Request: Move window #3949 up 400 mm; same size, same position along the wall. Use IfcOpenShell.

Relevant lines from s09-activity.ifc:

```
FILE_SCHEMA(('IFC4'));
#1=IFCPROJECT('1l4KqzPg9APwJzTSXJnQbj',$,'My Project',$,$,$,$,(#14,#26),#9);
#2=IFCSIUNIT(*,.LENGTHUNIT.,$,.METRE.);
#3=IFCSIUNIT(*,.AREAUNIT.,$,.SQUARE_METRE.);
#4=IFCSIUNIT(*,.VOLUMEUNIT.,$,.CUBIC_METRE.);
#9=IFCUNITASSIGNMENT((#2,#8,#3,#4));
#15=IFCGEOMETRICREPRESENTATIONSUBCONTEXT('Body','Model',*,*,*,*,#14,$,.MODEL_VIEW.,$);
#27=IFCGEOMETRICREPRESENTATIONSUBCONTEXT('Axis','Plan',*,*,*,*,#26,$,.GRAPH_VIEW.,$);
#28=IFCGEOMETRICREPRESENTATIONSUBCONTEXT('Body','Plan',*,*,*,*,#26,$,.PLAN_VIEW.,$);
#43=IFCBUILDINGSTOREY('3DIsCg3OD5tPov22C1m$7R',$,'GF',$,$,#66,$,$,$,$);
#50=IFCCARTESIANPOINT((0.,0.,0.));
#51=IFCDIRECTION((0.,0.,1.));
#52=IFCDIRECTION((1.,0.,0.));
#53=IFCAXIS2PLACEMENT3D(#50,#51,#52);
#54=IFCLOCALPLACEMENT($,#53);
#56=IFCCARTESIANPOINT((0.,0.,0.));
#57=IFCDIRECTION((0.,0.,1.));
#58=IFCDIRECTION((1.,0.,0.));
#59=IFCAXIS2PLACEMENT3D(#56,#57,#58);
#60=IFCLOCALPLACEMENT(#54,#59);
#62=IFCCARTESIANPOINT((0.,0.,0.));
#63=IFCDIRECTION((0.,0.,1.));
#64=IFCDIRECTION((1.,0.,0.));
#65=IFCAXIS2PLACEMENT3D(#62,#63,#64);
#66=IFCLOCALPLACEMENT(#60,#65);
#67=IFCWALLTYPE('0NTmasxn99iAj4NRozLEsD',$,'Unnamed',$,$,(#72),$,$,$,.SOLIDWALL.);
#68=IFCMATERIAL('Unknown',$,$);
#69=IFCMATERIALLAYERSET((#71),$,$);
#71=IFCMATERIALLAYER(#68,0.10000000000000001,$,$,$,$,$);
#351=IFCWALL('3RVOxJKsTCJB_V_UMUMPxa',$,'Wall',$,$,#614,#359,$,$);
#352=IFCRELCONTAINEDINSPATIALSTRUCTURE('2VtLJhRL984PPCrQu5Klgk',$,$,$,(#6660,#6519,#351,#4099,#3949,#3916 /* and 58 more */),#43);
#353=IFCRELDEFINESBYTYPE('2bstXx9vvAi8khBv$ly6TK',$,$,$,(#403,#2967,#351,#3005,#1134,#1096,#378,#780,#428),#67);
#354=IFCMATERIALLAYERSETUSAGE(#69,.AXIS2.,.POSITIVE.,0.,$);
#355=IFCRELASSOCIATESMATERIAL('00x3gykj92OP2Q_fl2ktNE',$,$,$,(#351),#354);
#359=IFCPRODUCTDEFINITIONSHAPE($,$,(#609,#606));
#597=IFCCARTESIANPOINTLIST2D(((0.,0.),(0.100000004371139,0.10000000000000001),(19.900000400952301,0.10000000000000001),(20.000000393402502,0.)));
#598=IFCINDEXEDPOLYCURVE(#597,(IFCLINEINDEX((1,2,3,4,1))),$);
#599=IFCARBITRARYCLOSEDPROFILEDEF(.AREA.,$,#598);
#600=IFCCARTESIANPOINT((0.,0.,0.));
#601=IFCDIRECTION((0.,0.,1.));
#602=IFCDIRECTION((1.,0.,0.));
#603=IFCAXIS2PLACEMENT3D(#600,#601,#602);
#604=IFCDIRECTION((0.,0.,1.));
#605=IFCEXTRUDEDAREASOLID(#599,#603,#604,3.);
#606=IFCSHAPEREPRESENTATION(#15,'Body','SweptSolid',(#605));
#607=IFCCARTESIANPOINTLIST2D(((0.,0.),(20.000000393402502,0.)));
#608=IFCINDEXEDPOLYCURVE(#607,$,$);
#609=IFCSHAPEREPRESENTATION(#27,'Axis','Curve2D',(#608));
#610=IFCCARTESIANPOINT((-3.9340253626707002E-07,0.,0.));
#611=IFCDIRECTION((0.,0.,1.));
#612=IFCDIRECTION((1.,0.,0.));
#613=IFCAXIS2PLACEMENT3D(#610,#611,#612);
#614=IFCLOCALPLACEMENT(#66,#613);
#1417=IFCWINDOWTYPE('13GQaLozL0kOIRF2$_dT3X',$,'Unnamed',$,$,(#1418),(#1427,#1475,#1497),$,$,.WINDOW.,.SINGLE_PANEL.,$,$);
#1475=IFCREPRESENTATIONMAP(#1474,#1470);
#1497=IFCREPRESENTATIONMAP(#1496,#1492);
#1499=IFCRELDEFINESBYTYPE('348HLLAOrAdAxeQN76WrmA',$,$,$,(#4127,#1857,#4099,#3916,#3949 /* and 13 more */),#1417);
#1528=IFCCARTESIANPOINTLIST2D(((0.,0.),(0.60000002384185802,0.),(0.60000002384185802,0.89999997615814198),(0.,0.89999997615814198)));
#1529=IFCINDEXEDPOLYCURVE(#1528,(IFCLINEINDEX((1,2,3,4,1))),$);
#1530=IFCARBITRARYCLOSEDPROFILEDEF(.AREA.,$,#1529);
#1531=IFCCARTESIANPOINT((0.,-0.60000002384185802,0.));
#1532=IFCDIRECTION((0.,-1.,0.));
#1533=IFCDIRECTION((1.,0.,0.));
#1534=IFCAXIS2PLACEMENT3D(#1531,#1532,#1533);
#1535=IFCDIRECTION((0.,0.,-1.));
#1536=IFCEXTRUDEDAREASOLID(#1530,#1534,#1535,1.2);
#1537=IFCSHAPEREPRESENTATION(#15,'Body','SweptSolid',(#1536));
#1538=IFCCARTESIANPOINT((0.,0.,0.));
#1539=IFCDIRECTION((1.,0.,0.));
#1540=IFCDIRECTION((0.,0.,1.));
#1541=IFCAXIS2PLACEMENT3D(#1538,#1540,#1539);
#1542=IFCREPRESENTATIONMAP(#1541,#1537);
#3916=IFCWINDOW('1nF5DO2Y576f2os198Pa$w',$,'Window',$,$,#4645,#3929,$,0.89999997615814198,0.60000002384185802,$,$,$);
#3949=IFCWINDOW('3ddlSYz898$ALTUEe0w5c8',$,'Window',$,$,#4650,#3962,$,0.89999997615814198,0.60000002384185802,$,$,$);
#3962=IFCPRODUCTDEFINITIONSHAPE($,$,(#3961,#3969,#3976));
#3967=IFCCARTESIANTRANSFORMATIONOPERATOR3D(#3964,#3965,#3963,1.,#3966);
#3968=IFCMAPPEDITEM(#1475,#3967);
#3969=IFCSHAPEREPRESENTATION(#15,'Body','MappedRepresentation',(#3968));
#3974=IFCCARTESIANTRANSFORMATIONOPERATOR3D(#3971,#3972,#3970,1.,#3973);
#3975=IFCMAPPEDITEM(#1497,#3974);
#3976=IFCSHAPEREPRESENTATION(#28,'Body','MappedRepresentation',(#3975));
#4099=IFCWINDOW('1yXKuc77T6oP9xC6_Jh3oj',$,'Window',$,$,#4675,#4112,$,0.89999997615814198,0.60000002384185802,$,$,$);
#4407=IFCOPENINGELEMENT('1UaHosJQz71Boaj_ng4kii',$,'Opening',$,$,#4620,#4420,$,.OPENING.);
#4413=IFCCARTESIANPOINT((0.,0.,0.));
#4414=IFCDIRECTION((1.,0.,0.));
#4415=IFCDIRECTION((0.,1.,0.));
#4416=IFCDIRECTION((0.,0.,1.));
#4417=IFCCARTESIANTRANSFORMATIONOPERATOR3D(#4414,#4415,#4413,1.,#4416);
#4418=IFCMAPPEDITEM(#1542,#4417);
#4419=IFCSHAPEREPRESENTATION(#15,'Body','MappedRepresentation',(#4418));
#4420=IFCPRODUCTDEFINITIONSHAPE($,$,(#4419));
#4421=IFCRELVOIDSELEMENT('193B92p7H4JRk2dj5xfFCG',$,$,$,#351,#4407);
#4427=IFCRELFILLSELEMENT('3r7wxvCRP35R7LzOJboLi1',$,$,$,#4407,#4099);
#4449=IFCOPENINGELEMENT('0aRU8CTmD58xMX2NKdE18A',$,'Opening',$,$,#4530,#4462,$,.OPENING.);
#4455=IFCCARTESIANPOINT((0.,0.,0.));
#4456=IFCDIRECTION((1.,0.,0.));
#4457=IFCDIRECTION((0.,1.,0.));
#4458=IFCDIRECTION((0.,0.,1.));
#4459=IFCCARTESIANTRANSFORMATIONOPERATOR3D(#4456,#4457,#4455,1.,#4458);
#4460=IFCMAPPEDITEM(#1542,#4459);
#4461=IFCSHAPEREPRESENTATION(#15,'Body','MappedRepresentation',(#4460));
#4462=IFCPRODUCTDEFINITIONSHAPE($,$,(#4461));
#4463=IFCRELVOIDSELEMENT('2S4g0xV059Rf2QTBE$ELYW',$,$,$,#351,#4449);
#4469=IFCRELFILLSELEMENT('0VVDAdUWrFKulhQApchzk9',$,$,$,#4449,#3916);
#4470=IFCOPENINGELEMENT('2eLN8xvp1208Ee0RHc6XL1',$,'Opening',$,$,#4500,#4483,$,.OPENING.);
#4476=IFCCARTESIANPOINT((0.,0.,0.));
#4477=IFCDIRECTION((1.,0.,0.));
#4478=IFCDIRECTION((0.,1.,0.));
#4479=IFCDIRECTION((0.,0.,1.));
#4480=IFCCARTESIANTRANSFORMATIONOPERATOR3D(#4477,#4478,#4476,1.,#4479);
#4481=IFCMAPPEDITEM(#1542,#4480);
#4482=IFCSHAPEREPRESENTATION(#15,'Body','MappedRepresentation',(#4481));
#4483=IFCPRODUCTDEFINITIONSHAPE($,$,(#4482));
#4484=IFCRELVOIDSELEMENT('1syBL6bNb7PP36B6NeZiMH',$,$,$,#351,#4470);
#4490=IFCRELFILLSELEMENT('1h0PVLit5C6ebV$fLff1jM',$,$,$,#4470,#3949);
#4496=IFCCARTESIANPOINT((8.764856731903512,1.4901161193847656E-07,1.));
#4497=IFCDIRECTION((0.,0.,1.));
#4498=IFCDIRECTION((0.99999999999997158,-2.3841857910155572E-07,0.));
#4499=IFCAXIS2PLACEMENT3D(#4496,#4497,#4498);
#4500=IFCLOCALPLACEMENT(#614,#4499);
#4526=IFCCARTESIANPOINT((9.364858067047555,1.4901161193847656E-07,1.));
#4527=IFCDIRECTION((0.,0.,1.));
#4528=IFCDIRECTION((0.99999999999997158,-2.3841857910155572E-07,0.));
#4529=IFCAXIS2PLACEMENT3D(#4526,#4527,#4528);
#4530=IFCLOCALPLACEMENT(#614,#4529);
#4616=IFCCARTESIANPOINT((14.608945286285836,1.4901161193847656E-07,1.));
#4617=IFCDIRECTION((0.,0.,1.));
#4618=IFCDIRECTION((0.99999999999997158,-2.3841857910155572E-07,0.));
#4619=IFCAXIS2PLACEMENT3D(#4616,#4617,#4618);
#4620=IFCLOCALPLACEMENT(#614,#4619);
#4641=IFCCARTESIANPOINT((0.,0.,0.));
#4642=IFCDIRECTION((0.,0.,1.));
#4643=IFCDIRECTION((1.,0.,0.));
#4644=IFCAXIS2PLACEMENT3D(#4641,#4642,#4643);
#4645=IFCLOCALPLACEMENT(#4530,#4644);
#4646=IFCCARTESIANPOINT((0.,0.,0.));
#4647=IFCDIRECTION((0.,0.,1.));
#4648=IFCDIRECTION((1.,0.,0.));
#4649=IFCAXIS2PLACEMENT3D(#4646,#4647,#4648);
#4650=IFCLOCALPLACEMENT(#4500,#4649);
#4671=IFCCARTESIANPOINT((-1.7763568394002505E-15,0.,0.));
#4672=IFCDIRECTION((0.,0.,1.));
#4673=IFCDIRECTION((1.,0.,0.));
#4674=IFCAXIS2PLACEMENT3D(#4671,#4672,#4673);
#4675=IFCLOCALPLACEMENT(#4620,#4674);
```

```python
import numpy as np
import ifcopenshell
import ifcopenshell.api.geometry
import ifcopenshell.util.placement
import ifcopenshell.util.unit

model = ifcopenshell.open("s09-activity.ifc")
unit_scale = ifcopenshell.util.unit.calculate_unit_scale(model)

window = model.by_guid("3ddlSYz898$ALTUEe0w5c8")
opening = window.FillsVoids[0].RelatingOpeningElement
dz = 0.4 / unit_scale

shift = np.array([0.0, 0.0, dz])
# The window is placed relative to its opening, so it follows when the opening moves.
matrix = ifcopenshell.util.placement.get_local_placement(opening.ObjectPlacement)
matrix[:3, 3] += shift
ifcopenshell.api.geometry.edit_object_placement(
    model, product=opening, matrix=matrix, is_si=False, should_transform_children=True
)

print(f"moved by {dz * unit_scale:+.3f} m")

model.write("s09-activity_updated.ifc")
```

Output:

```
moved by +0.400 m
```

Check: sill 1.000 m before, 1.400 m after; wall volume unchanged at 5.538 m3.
